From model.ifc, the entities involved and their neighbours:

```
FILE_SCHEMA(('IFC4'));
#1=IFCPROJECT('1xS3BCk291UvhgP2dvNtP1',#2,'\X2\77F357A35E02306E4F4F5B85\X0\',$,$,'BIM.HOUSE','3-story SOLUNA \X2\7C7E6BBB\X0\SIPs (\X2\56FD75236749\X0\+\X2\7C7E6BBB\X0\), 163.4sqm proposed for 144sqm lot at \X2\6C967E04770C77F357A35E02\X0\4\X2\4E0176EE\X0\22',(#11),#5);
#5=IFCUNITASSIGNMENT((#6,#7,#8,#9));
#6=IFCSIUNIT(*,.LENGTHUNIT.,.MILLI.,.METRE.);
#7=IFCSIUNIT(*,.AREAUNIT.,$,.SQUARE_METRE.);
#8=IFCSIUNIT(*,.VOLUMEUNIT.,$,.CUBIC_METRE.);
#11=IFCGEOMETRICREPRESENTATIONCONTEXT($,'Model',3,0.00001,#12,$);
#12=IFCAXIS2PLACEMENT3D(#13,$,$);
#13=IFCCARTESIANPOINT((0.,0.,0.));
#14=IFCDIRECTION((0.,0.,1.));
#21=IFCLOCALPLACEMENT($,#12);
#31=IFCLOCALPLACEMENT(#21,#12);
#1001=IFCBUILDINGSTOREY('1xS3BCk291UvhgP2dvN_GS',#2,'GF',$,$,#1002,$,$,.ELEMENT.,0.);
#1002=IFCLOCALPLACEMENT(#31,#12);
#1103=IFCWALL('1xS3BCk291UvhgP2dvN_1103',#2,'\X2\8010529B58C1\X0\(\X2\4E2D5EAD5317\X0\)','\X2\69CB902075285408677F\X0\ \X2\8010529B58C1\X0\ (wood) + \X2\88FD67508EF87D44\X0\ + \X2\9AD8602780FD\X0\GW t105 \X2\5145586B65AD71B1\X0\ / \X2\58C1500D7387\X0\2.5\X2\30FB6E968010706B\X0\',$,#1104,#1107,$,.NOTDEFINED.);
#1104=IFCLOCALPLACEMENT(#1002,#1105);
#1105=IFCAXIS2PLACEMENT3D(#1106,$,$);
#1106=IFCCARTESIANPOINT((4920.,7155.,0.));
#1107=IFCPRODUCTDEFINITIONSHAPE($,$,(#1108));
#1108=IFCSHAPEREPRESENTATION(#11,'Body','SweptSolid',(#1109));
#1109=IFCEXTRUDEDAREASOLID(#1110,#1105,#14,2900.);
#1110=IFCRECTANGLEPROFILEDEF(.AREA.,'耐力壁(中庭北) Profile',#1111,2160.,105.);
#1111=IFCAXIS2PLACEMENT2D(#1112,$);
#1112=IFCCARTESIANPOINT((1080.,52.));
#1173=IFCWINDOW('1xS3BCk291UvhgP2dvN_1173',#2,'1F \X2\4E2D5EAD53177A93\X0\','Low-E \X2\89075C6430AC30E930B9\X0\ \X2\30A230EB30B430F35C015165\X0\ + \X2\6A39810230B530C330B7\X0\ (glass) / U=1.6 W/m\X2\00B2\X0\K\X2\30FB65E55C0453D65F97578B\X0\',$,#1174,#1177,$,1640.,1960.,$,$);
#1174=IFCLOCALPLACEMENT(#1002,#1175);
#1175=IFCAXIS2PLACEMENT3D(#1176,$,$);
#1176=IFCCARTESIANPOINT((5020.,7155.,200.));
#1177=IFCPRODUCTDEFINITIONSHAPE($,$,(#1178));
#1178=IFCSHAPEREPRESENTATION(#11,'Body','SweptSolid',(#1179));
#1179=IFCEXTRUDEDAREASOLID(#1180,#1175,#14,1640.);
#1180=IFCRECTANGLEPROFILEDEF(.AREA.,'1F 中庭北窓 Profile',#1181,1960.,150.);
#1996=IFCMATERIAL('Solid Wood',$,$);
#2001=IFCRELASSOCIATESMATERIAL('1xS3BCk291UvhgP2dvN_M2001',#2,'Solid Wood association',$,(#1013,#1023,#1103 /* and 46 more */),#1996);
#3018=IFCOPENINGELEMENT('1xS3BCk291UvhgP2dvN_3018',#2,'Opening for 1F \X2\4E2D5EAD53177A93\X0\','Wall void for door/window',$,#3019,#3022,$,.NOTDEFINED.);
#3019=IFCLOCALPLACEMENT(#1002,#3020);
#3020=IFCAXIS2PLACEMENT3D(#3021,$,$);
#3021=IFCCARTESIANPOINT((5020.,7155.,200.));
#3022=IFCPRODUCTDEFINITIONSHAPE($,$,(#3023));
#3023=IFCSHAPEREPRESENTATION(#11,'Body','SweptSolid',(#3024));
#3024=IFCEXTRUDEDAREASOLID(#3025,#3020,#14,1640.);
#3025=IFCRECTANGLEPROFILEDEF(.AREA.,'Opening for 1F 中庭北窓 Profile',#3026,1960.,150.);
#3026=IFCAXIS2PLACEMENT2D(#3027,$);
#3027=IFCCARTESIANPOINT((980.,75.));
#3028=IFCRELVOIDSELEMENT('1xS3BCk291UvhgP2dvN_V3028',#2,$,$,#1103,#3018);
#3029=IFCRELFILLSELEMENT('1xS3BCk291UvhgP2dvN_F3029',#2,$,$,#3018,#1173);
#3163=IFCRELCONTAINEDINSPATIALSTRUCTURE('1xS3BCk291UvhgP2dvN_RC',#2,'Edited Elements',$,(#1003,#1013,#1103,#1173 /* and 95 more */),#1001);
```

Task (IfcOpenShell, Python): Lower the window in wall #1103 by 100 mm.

```python
import numpy as np
import ifcopenshell
import ifcopenshell.api.geometry
import ifcopenshell.util.placement
import ifcopenshell.util.unit

model = ifcopenshell.open("model.ifc")
unit_scale = ifcopenshell.util.unit.calculate_unit_scale(model)

window = model.by_guid("1xS3BCk291UvhgP2dvN_1173")
opening = window.FillsVoids[0].RelatingOpeningElement
dz = -0.1 / unit_scale

shift = np.array([0.0, 0.0, dz])
# The window is not placed relative to its opening, so move both.
for product in (opening, window):
    matrix = ifcopenshell.util.placement.get_local_placement(product.ObjectPlacement)
    matrix[:3, 3] += shift
    ifcopenshell.api.geometry.edit_object_placement(model, product=product, matrix=matrix, is_si=False)

print(f"moved by {dz * unit_scale:+.3f} m")

model.write("model_edited.ifc")
```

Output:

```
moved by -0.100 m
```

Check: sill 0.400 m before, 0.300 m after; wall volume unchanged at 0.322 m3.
